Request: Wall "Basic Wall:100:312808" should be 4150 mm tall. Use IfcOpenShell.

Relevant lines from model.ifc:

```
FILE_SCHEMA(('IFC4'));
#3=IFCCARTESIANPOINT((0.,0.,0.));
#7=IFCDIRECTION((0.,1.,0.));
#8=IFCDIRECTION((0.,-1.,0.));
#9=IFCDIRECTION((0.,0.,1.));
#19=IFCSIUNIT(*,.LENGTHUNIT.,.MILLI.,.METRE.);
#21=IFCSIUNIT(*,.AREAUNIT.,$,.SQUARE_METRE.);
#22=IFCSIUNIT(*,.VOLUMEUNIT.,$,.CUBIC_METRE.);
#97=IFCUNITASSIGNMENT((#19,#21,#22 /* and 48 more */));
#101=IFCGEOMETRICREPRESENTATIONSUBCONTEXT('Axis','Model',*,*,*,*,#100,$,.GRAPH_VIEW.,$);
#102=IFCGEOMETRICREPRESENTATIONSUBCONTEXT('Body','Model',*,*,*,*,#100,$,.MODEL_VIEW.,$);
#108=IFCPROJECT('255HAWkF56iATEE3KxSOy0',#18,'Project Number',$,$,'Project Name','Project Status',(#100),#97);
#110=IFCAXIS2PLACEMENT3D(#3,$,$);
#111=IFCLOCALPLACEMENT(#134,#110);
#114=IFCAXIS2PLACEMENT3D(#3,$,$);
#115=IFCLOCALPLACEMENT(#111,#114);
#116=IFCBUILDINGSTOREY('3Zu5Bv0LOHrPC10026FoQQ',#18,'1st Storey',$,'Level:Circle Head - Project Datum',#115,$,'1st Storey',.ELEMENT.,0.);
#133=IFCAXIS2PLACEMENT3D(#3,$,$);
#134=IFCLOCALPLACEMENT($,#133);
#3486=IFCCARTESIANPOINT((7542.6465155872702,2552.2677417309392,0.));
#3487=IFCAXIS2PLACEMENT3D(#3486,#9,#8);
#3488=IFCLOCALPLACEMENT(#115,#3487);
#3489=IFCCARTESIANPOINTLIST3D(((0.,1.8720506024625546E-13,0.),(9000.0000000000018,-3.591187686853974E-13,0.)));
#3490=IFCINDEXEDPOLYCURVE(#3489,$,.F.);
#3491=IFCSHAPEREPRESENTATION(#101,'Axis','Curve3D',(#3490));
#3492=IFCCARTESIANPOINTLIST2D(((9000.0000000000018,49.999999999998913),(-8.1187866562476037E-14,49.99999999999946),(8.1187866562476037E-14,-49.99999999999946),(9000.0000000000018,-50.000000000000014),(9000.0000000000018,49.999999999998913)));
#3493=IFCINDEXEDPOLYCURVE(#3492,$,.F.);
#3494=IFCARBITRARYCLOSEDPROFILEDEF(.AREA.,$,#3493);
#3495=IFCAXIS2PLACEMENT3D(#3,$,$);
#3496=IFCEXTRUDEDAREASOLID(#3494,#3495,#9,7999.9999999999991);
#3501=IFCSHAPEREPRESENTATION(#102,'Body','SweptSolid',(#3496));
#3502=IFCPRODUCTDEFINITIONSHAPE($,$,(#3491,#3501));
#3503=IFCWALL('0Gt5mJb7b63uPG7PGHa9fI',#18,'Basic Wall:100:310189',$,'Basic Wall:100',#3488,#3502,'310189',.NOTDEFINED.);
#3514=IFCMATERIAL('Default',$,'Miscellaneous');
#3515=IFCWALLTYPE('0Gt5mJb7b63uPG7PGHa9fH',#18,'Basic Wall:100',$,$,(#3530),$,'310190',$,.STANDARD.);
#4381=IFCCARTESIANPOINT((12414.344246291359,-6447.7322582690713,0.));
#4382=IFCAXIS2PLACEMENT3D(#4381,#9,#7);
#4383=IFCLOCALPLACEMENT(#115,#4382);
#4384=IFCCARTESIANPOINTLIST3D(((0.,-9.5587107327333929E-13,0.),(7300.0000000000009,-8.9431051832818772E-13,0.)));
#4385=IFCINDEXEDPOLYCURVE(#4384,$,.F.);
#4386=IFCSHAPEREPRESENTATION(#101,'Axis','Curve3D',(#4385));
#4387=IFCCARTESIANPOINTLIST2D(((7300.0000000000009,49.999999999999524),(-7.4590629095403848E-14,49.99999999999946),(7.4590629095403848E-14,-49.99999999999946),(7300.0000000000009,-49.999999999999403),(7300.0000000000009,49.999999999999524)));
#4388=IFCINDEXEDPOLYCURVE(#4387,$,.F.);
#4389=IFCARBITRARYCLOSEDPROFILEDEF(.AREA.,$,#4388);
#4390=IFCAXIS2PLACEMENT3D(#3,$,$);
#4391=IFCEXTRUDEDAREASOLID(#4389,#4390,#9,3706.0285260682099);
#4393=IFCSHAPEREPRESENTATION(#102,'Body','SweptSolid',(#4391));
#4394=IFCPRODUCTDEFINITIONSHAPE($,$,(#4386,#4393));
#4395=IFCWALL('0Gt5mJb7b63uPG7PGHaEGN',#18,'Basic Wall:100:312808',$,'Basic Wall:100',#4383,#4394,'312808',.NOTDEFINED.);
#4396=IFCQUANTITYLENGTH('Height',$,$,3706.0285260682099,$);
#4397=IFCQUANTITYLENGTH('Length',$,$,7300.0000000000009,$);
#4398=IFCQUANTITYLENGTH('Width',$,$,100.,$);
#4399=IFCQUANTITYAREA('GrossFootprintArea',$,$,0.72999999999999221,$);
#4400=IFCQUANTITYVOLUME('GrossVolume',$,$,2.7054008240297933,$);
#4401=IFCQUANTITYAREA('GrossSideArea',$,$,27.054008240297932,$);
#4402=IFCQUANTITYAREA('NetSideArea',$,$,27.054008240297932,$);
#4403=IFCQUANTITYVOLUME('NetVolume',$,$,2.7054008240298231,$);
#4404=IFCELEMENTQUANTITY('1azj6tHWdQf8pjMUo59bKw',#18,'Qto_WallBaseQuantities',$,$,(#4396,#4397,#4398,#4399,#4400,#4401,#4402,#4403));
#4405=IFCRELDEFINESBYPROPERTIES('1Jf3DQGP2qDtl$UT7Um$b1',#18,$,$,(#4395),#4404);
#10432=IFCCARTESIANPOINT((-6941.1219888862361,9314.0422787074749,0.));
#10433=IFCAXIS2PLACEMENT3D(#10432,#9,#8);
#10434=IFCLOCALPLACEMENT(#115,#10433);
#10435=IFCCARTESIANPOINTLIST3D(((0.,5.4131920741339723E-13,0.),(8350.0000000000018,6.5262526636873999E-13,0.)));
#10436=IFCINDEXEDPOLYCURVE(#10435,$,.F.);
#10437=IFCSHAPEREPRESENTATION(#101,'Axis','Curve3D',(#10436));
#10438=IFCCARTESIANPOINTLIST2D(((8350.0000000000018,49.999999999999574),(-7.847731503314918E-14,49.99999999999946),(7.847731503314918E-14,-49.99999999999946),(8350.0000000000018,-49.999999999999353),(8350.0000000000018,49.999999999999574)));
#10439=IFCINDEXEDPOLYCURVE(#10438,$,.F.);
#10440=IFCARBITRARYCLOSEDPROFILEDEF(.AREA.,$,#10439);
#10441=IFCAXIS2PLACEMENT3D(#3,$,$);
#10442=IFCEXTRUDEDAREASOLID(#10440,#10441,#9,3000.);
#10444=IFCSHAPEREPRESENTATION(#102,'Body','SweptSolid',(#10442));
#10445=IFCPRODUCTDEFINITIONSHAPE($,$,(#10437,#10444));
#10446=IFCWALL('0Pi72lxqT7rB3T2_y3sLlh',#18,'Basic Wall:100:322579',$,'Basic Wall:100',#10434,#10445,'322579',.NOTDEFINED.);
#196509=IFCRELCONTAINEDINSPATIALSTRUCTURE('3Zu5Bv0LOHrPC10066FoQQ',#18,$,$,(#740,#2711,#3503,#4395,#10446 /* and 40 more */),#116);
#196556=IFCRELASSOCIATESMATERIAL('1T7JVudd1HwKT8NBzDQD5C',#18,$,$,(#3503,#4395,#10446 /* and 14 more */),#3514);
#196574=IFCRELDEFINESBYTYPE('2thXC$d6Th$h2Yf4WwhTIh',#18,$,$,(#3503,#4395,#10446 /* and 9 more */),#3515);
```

```python
import ifcopenshell
import ifcopenshell.api.pset
import ifcopenshell.geom
import ifcopenshell.util.element
import ifcopenshell.util.representation
import ifcopenshell.util.shape
import ifcopenshell.util.unit

model = ifcopenshell.open("model.ifc")
unit_scale = ifcopenshell.util.unit.calculate_unit_scale(model)
area_scale = ifcopenshell.util.unit.calculate_unit_scale(model, "AREAUNIT")
volume_scale = ifcopenshell.util.unit.calculate_unit_scale(model, "VOLUMEUNIT")
settings = ifcopenshell.geom.settings()


def volume(element):
    """Net volume in cubic metres, openings subtracted."""
    shape = ifcopenshell.geom.create_shape(settings, element)
    return ifcopenshell.util.shape.get_volume(shape.geometry)


wall = model.by_guid("0Gt5mJb7b63uPG7PGHaEGN")
before = volume(wall)

body = ifcopenshell.util.representation.get_representation(wall, "Model", "Body")
solid = body.Items[0]
old_height = solid.Depth
solid.Depth = 4.15 / unit_scale
after = volume(wall)
thickness = 0.1  # wall thickness in metres

# Update the stored height, areas and volumes.
qto = model.by_id(ifcopenshell.util.element.get_pset(wall, "Qto_WallBaseQuantities", should_inherit=False)["id"])
ifcopenshell.api.pset.edit_qto(model, qto=qto, properties={
    "Height": solid.Depth,
    "GrossVolume": ifcopenshell.util.element.get_pset(wall, "Qto_WallBaseQuantities", "GrossVolume") * solid.Depth / old_height,
    "GrossSideArea": ifcopenshell.util.element.get_pset(wall, "Qto_WallBaseQuantities", "GrossSideArea") * solid.Depth / old_height,
    "NetSideArea": after / thickness / area_scale,
    "NetVolume": after / volume_scale,
})

print(f"height {old_height:g} -> {solid.Depth:g}, volume {before:.3f} -> {after:.3f} m3")

model.write("model_rev.ifc")
```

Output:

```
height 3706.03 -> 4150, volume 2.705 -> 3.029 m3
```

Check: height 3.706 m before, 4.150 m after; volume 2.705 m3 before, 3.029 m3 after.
